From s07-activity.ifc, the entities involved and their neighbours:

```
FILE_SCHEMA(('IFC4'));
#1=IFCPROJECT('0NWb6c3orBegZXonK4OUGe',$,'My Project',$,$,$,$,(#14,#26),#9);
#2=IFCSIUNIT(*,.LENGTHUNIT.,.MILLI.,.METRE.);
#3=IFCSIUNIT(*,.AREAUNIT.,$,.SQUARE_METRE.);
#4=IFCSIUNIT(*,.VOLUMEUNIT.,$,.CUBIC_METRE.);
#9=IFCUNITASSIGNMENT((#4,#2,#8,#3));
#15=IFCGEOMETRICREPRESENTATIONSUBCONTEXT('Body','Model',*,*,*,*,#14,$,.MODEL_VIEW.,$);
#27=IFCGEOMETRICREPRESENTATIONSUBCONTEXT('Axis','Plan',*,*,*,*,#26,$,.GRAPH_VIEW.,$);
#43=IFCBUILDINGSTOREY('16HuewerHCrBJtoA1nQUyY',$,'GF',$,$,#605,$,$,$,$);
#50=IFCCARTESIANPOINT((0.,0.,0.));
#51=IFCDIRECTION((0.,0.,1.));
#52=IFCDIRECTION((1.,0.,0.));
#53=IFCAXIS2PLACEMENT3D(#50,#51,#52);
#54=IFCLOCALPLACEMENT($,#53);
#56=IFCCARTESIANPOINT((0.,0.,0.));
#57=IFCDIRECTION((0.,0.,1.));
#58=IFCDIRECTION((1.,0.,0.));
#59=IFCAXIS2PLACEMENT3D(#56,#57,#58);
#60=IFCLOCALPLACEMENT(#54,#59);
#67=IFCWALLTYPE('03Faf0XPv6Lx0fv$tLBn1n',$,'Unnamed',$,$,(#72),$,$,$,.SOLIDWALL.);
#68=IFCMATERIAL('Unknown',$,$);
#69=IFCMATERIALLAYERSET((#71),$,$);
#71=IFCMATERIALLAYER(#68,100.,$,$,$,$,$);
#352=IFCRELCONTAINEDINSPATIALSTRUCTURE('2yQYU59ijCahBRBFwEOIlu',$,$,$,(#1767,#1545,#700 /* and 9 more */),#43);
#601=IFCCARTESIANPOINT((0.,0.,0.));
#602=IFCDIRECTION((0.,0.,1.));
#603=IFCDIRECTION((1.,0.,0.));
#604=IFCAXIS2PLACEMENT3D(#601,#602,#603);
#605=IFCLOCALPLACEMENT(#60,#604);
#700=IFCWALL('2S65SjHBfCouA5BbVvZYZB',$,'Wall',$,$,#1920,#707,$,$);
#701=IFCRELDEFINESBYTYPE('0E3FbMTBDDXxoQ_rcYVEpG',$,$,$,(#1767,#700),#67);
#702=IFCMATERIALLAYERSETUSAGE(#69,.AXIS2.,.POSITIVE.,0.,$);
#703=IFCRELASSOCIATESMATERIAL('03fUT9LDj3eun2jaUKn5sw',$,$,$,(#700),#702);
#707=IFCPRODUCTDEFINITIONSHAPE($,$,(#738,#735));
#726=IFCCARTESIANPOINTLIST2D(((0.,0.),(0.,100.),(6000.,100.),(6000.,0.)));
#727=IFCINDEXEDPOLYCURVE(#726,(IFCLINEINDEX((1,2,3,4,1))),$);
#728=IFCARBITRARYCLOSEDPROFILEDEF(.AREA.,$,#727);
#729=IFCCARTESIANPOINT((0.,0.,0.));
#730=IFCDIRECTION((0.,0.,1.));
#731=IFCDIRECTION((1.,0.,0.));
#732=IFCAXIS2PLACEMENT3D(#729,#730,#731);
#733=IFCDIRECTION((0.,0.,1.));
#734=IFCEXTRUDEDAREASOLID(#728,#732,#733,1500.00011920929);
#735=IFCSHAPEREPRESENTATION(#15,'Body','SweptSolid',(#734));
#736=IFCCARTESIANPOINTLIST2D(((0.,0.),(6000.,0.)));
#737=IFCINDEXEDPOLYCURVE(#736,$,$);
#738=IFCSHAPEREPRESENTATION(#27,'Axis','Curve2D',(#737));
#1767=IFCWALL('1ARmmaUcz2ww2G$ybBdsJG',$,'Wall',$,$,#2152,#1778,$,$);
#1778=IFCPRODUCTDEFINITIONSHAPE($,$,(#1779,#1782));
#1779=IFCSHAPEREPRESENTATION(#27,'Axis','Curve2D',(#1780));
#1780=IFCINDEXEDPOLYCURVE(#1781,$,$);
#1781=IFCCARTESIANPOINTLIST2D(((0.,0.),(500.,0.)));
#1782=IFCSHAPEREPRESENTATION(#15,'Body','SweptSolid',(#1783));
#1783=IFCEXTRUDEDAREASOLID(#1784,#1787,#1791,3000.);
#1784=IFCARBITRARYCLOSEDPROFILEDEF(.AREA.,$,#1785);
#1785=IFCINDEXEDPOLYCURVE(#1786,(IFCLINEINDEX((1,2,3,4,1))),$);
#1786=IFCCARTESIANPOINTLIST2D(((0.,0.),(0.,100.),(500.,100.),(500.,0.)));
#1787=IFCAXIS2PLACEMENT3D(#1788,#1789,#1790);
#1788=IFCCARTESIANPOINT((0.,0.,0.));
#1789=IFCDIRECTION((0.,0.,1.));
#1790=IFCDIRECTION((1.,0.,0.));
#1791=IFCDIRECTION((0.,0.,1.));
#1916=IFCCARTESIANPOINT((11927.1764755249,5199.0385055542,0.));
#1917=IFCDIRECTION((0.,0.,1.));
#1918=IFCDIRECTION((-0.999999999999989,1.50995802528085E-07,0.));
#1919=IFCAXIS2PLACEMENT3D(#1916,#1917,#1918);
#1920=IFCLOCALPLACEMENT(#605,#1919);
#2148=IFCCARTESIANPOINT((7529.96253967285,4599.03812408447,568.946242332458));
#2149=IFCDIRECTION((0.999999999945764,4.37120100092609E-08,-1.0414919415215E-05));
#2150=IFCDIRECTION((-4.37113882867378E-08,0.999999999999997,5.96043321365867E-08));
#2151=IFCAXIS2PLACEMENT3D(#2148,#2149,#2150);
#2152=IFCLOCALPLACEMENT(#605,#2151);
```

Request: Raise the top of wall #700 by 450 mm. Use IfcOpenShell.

```python
import ifcopenshell
import ifcopenshell.geom
import ifcopenshell.util.representation
import ifcopenshell.util.shape

model = ifcopenshell.open("s07-activity.ifc")
settings = ifcopenshell.geom.settings()


def volume(element):
    """Net volume in cubic metres, openings subtracted."""
    shape = ifcopenshell.geom.create_shape(settings, element)
    return ifcopenshell.util.shape.get_volume(shape.geometry)


wall = model.by_id(700)
before = volume(wall)

body = ifcopenshell.util.representation.get_representation(wall, "Model", "Body")
solid = body.Items[0]
old_height = solid.Depth
solid.Depth += 450.0
after = volume(wall)

print(f"height {old_height:g} -> {solid.Depth:g}, volume {before:.3f} -> {after:.3f} m3")

model.write("s07-activity_v2.ifc")
```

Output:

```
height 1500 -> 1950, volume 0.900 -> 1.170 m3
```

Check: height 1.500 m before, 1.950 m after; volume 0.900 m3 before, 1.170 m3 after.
